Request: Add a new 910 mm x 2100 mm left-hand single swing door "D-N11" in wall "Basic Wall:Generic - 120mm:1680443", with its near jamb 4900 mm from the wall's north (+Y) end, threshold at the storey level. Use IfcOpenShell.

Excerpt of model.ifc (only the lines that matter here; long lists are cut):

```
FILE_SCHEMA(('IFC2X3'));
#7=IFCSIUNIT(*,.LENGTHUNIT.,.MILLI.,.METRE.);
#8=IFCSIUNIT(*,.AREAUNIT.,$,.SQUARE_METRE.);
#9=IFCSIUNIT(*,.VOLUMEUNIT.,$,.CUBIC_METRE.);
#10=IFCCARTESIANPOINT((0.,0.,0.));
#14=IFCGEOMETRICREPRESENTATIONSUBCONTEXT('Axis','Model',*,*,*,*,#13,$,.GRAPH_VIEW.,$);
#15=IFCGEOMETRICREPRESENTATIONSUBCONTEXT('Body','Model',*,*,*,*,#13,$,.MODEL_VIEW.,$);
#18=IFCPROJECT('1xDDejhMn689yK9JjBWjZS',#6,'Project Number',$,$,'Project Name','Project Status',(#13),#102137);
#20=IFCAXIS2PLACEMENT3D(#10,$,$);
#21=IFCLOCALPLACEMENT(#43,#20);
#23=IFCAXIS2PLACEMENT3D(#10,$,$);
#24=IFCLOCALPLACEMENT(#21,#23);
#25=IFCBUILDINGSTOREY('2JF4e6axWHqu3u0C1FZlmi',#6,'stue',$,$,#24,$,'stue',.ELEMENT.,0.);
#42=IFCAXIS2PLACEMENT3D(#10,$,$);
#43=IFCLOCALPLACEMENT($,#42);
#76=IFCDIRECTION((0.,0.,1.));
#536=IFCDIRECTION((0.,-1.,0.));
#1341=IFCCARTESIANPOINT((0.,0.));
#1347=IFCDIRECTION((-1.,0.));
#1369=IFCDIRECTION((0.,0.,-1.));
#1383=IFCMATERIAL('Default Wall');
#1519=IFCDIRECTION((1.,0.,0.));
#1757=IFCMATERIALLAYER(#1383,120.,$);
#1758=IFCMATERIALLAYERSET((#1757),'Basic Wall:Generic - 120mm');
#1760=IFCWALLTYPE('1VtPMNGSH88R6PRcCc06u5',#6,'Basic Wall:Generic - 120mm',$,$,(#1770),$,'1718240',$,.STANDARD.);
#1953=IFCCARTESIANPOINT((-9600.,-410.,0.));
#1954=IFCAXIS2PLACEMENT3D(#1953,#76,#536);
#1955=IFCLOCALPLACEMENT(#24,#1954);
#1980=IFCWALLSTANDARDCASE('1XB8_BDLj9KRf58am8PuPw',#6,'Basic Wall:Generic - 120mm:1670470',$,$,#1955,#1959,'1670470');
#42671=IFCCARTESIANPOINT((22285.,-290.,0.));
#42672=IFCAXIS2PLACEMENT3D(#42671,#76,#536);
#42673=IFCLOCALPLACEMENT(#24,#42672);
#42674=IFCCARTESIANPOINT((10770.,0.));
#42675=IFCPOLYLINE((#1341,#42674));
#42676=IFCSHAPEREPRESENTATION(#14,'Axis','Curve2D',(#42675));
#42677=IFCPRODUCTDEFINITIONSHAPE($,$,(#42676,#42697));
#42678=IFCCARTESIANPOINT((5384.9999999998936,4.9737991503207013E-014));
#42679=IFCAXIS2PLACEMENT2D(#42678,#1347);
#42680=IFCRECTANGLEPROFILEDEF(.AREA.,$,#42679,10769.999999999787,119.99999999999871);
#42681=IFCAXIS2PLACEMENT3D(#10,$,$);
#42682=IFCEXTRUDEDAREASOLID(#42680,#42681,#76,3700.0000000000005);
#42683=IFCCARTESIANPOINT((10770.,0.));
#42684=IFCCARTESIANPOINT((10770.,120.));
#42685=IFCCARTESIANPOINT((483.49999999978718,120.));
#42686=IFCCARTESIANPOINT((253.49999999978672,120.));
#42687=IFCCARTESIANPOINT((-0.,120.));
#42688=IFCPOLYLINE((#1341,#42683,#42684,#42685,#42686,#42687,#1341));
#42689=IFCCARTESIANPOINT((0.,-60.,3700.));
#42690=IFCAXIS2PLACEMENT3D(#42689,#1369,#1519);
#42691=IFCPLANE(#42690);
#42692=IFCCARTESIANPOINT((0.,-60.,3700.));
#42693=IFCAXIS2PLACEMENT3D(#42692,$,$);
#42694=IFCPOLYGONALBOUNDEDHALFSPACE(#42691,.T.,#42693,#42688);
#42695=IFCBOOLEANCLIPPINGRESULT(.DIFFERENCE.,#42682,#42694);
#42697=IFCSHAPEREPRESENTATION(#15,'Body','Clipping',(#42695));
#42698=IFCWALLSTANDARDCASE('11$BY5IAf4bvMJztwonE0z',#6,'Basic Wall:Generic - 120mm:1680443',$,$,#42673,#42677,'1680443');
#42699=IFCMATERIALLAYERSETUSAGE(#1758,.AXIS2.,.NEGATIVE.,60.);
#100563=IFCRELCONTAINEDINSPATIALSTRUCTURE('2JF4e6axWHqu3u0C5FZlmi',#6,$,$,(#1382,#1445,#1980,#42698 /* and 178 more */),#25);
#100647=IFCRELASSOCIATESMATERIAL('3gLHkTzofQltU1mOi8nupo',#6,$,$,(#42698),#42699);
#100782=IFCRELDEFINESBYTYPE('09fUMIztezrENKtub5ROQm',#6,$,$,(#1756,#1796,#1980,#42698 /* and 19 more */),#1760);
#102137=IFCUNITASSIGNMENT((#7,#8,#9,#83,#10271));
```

```python
import numpy as np
import ifcopenshell
import ifcopenshell.api.feature
import ifcopenshell.api.geometry
import ifcopenshell.api.root
import ifcopenshell.api.spatial
import ifcopenshell.api.type
import ifcopenshell.geom
import ifcopenshell.util.element
import ifcopenshell.util.placement
import ifcopenshell.util.representation
import ifcopenshell.util.shape
import ifcopenshell.util.unit

model = ifcopenshell.open("model.ifc")
unit_scale = ifcopenshell.util.unit.calculate_unit_scale(model)
settings = ifcopenshell.geom.settings()


def volume(element):
    """Net volume in cubic metres, openings subtracted."""
    shape = ifcopenshell.geom.create_shape(settings, element)
    return ifcopenshell.util.shape.get_volume(shape.geometry)


wall = model.by_guid("11$BY5IAf4bvMJztwonE0z")
storey = ifcopenshell.util.element.get_container(wall, ifc_class="IfcBuildingStorey")
context = ifcopenshell.util.representation.get_context(model, "Model", "Body", "MODEL_VIEW")
before = volume(wall)

width, height, from_end, sill = 0.91, 2.1, 4.9, 0.0  # metres

# The wall runs along its own X axis, and the end named is its -X end.
wall_shape = ifcopenshell.geom.create_shape(settings, wall)
x, y, z = ifcopenshell.util.shape.get_vertices(wall_shape.geometry).T
start = x.min() + from_end
face, thickness = float(y.min()), float(y.max() - y.min())
wall_matrix = ifcopenshell.util.placement.get_local_placement(wall.ObjectPlacement)
level = ifcopenshell.util.placement.get_local_placement(storey.ObjectPlacement)[2, 3]


def in_wall(x, y):
    """Placement at x, y metres in the wall's axes, at sill height."""
    matrix = wall_matrix.copy()
    matrix[:, 3] = wall_matrix @ np.array([x / unit_scale, y / unit_scale, 0.0, 1.0])
    matrix[2, 3] = level + sill / unit_scale
    return matrix


# Opening: a box that overshoots both wall faces by 50 mm.
opening = ifcopenshell.api.root.create_entity(model, ifc_class="IfcOpeningElement")
box = ifcopenshell.api.geometry.add_wall_representation(
    model, context=context, length=width, height=height, thickness=thickness + 0.1
)
ifcopenshell.api.geometry.assign_representation(model, product=opening, representation=box)
ifcopenshell.api.geometry.edit_object_placement(model, product=opening, matrix=in_wall(start, face - 0.05), is_si=False)
ifcopenshell.api.feature.add_feature(model, feature=opening, element=wall)

door = ifcopenshell.api.root.create_entity(model, ifc_class="IfcDoor", name="D-N11")
door.OverallWidth, door.OverallHeight = width / unit_scale, height / unit_scale
body = ifcopenshell.api.geometry.add_door_representation(
    model,
    context=context,
    overall_width=door.OverallWidth,
    overall_height=door.OverallHeight,
    operation_type="SINGLE_SWING_LEFT",
    lining_properties={"LiningDepth": thickness / unit_scale, "ThresholdDepth": thickness / unit_scale},
)
ifcopenshell.api.geometry.assign_representation(model, product=door, representation=body)
ifcopenshell.api.spatial.assign_container(model, products=[door], relating_structure=storey)
fills = ifcopenshell.api.feature.add_filling(model, opening=opening, element=door)
fills.OwnerHistory = door.OwnerHistory  # required in IFC2X3

# IFC2X3 keeps the operation on the door style.
style = ifcopenshell.api.root.create_entity(model, ifc_class="IfcDoorStyle", name="D-N11")
style.OperationType, style.ConstructionType = "SINGLE_SWING_LEFT", "NOTDEFINED"
style.ParameterTakesPrecedence = style.Sizeable = False
ifcopenshell.api.type.assign_type(model, related_objects=[door], relating_type=style)

# The lining spans the wall, so the door starts at the wall face.
ifcopenshell.api.geometry.edit_object_placement(model, product=door, matrix=in_wall(start, face), is_si=False)

after = volume(wall)

print(f"wall volume {before:.3f} -> {after:.3f} m3")

model.write("model_updated.ifc")
```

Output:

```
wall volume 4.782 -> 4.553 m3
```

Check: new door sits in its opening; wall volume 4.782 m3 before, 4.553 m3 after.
